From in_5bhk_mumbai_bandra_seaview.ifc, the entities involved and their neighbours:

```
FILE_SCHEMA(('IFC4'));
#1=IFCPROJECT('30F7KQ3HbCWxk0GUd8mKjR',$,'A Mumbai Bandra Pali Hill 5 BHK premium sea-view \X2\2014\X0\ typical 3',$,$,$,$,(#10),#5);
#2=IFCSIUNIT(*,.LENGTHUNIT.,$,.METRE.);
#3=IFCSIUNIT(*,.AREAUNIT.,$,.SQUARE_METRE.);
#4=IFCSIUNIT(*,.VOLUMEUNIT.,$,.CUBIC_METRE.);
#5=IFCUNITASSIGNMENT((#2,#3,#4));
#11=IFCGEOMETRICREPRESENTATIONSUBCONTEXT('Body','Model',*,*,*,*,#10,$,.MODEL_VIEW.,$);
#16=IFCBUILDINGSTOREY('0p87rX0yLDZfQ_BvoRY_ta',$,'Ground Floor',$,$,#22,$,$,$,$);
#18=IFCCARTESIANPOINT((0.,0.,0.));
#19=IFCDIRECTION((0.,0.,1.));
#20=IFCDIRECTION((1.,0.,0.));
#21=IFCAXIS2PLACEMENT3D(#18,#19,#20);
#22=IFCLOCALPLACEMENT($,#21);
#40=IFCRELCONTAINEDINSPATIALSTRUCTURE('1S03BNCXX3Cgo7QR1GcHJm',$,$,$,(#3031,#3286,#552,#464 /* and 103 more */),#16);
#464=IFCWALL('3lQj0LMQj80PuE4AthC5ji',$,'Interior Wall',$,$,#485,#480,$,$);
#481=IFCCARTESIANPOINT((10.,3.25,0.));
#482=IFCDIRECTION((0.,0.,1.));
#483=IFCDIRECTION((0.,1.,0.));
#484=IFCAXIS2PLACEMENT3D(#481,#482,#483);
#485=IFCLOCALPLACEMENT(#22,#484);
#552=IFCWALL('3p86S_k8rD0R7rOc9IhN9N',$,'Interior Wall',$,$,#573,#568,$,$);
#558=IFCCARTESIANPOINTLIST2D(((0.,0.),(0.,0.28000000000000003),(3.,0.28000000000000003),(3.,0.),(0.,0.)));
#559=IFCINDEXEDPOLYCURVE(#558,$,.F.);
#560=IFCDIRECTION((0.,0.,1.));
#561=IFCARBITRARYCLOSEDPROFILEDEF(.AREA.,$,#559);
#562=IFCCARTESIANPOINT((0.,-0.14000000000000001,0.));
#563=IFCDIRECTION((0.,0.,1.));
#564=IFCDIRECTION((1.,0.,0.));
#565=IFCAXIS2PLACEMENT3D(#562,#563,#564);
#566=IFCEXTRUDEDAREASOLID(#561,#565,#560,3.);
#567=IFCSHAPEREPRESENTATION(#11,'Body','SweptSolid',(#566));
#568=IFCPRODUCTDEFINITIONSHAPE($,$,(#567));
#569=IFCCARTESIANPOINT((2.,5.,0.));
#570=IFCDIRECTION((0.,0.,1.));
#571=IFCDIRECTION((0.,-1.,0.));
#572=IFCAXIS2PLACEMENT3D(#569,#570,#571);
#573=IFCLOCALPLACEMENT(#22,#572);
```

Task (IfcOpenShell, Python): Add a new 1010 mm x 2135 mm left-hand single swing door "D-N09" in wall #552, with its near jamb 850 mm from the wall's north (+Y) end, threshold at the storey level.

```python
import numpy as np
import ifcopenshell
import ifcopenshell.api.feature
import ifcopenshell.api.geometry
import ifcopenshell.api.root
import ifcopenshell.api.spatial
import ifcopenshell.geom
import ifcopenshell.util.element
import ifcopenshell.util.placement
import ifcopenshell.util.representation
import ifcopenshell.util.shape
import ifcopenshell.util.unit

model = ifcopenshell.open("in_5bhk_mumbai_bandra_seaview.ifc")
unit_scale = ifcopenshell.util.unit.calculate_unit_scale(model)
settings = ifcopenshell.geom.settings()


def volume(element):
    """Net volume in cubic metres, openings subtracted."""
    shape = ifcopenshell.geom.create_shape(settings, element)
    return ifcopenshell.util.shape.get_volume(shape.geometry)


wall = model.by_guid("3p86S_k8rD0R7rOc9IhN9N")
storey = ifcopenshell.util.element.get_container(wall, ifc_class="IfcBuildingStorey")
context = ifcopenshell.util.representation.get_context(model, "Model", "Body", "MODEL_VIEW")
before = volume(wall)

width, height, from_end, sill = 1.01, 2.135, 0.85, 0.0  # metres

# The wall runs along its own X axis, and the end named is its -X end.
wall_shape = ifcopenshell.geom.create_shape(settings, wall)
x, y, z = ifcopenshell.util.shape.get_vertices(wall_shape.geometry).T
start = x.min() + from_end
face, thickness = float(y.min()), float(y.max() - y.min())
wall_matrix = ifcopenshell.util.placement.get_local_placement(wall.ObjectPlacement)
level = ifcopenshell.util.placement.get_local_placement(storey.ObjectPlacement)[2, 3]


def in_wall(x, y):
    """Placement at x, y metres in the wall's axes, at sill height."""
    matrix = wall_matrix.copy()
    matrix[:, 3] = wall_matrix @ np.array([x / unit_scale, y / unit_scale, 0.0, 1.0])
    matrix[2, 3] = level + sill / unit_scale
    return matrix


# Opening: a box that overshoots both wall faces by 50 mm.
opening = ifcopenshell.api.root.create_entity(model, ifc_class="IfcOpeningElement", predefined_type="OPENING")
box = ifcopenshell.api.geometry.add_wall_representation(
    model, context=context, length=width, height=height, thickness=thickness + 0.1
)
ifcopenshell.api.geometry.assign_representation(model, product=opening, representation=box)
ifcopenshell.api.geometry.edit_object_placement(model, product=opening, matrix=in_wall(start, face - 0.05), is_si=False)
ifcopenshell.api.feature.add_feature(model, feature=opening, element=wall)

door = ifcopenshell.api.root.create_entity(model, ifc_class="IfcDoor", name="D-N09", predefined_type="DOOR")
door.OverallWidth, door.OverallHeight = width / unit_scale, height / unit_scale
door.OperationType = "SINGLE_SWING_LEFT"
body = ifcopenshell.api.geometry.add_door_representation(
    model,
    context=context,
    overall_width=door.OverallWidth,
    overall_height=door.OverallHeight,
    operation_type="SINGLE_SWING_LEFT",
    lining_properties={"LiningDepth": thickness / unit_scale, "ThresholdDepth": thickness / unit_scale},
)
ifcopenshell.api.geometry.assign_representation(model, product=door, representation=body)
ifcopenshell.api.spatial.assign_container(model, products=[door], relating_structure=storey)
ifcopenshell.api.feature.add_filling(model, opening=opening, element=door)

# The lining spans the wall, so the door starts at the wall face.
ifcopenshell.api.geometry.edit_object_placement(model, product=door, matrix=in_wall(start, face), is_si=False)

after = volume(wall)

print(f"wall volume {before:.3f} -> {after:.3f} m3")

model.write("in_5bhk_mumbai_bandra_seaview_v2.ifc")
```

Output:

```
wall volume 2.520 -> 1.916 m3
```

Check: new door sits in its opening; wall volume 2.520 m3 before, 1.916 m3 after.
